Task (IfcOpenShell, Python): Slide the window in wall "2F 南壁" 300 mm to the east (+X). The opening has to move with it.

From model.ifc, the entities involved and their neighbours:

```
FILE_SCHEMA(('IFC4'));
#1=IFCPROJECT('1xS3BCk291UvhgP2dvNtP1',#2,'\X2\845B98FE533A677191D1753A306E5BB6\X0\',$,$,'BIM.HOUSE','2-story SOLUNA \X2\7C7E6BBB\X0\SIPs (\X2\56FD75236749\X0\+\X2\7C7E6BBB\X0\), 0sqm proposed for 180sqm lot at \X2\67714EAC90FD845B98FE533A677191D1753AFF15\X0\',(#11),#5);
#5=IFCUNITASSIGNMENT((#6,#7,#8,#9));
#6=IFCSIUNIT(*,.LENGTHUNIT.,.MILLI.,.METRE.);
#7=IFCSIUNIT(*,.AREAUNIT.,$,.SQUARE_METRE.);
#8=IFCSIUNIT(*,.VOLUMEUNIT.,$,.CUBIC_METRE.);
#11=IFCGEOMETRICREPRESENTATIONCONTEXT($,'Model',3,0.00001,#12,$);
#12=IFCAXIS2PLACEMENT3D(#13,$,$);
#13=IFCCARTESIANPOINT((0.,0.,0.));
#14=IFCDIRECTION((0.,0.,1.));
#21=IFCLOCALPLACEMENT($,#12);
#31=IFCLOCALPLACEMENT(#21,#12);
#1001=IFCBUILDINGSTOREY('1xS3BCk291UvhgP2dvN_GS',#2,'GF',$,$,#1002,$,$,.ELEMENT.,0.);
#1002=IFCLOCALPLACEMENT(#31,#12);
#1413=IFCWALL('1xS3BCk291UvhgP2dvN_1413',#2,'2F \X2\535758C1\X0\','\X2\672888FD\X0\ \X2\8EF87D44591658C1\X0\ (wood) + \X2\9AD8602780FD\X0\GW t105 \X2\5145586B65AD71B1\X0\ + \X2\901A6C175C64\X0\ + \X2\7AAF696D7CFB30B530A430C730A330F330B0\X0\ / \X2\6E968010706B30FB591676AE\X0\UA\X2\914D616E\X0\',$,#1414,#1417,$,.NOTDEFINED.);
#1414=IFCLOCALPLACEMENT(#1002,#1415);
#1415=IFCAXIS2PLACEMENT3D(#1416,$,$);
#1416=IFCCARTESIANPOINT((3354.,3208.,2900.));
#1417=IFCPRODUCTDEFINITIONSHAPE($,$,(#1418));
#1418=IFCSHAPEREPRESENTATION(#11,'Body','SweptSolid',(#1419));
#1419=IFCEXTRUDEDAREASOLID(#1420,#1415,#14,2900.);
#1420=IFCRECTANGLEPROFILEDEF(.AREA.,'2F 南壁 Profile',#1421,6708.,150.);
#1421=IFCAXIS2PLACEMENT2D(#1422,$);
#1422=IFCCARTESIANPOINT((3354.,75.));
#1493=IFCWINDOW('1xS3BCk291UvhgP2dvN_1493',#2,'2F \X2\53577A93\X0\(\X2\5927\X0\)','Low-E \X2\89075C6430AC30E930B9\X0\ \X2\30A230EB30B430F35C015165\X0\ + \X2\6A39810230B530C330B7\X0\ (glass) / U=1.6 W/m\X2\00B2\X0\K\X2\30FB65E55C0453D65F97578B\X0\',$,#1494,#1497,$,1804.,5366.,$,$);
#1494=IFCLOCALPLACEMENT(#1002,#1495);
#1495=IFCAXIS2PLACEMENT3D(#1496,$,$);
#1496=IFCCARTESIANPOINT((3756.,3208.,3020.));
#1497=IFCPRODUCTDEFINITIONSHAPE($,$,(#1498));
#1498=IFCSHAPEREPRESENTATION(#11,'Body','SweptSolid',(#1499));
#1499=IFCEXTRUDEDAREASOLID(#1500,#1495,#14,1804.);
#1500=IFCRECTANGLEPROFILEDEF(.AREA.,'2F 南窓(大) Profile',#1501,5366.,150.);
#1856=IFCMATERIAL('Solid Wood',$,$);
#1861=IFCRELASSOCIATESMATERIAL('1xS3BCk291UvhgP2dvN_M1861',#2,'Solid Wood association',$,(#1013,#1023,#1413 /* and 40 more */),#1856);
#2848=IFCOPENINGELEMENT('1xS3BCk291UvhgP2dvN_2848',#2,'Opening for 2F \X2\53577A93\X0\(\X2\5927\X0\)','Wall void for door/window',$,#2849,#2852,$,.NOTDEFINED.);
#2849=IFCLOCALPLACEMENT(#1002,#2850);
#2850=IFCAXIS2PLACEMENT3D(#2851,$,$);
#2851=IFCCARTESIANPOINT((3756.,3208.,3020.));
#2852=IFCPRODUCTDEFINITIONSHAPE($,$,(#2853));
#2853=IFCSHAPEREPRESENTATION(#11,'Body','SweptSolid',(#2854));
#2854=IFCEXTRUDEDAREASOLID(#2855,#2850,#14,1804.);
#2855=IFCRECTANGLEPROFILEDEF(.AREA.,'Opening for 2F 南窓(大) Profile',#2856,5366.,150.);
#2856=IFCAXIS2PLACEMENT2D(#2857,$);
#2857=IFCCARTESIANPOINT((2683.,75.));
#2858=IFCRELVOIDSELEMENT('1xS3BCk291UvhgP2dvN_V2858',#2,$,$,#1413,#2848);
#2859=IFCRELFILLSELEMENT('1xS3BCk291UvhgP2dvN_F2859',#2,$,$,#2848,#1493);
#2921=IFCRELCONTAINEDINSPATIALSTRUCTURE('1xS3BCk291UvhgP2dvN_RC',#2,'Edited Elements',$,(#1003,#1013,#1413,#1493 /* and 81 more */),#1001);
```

```python
import ifcopenshell
import ifcopenshell.api.geometry
import ifcopenshell.util.placement
import ifcopenshell.util.unit

model = ifcopenshell.open("model.ifc")
unit_scale = ifcopenshell.util.unit.calculate_unit_scale(model)

window = model.by_guid("1xS3BCk291UvhgP2dvN_1493")
opening = window.FillsVoids[0].RelatingOpeningElement
wall = opening.VoidsElements[0].RelatingBuildingElement

wall_matrix = ifcopenshell.util.placement.get_local_placement(wall.ObjectPlacement)
shift = wall_matrix[:3, 0] * 0.3 / unit_scale
before = ifcopenshell.util.placement.get_local_placement(window.ObjectPlacement)[:3, 3].copy()

# The window is not placed relative to its opening, so move both.
for product in (opening, window):
    matrix = ifcopenshell.util.placement.get_local_placement(product.ObjectPlacement)
    matrix[:3, 3] += shift
    ifcopenshell.api.geometry.edit_object_placement(model, product=product, matrix=matrix, is_si=False)

after = ifcopenshell.util.placement.get_local_placement(window.ObjectPlacement)[:3, 3]
print("window moved by", (after - before).round(3) + 0.0)

model.write("model-out.ifc")
```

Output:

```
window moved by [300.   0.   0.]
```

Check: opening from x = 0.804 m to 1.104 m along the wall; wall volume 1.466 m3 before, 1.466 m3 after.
